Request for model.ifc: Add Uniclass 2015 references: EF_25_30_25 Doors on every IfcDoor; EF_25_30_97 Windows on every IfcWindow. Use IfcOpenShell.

First a look at what the model holds.

```python
import ifcopenshell

model = ifcopenshell.open("model.ifc")
print(model.schema)
print("classifications:", [c.Name for c in model.by_type("IfcClassification")])
for ifc_class in ("IfcDoor", "IfcRoof", "IfcStair", "IfcWall", "IfcWindow"):
    print(ifc_class, len(model.by_type(ifc_class)))
```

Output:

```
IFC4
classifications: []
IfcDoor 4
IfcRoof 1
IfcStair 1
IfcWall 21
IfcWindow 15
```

```python
import ifcopenshell
import ifcopenshell.api.classification

model = ifcopenshell.open("model.ifc")

system = ifcopenshell.api.classification.add_classification(model, classification="Uniclass 2015")

codes = {
    "IfcDoor": ("EF_25_30_25", "Doors"),
    "IfcWindow": ("EF_25_30_97", "Windows"),
}
for ifc_class, (code, name) in codes.items():
    products = model.by_type(ifc_class)
    ifcopenshell.api.classification.add_reference(
        model, products=products, classification=system, identification=code, name=name
    )
    print(code, len(products))

model.write("model-out.ifc")
```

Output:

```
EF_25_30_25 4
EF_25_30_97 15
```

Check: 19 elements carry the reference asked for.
